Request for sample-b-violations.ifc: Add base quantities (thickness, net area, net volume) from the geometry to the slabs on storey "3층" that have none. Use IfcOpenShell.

First a look at what the model holds.

```python
import ifcopenshell
import ifcopenshell.util.element
import ifcopenshell.util.unit

model = ifcopenshell.open("sample-b-violations.ifc")
print(model.schema)
for unit_type in ("LENGTHUNIT", "AREAUNIT", "VOLUMEUNIT"):
    print(unit_type, ifcopenshell.util.unit.calculate_unit_scale(model, unit_type))
storey = next(s for s in model.by_type("IfcBuildingStorey") if s.Name == "3층")
slabs = [e for e in ifcopenshell.util.element.get_decomposition(storey) if e.is_a("IfcSlab")]
for e in sorted(slabs, key=lambda e: e.id()):
    print(e.id(), e.is_a(), e.Name, list(ifcopenshell.util.element.get_psets(e, qtos_only=True)), sep=" | ")
```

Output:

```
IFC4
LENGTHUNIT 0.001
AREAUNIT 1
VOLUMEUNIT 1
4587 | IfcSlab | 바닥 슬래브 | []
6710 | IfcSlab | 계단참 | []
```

```python
import ifcopenshell
import ifcopenshell.api.pset
import ifcopenshell.geom
import ifcopenshell.util.element
import ifcopenshell.util.shape
import ifcopenshell.util.unit

model = ifcopenshell.open("sample-b-violations.ifc")
unit_scale = ifcopenshell.util.unit.calculate_unit_scale(model)
area_scale = ifcopenshell.util.unit.calculate_unit_scale(model, "AREAUNIT")
volume_scale = ifcopenshell.util.unit.calculate_unit_scale(model, "VOLUMEUNIT")
settings = ifcopenshell.geom.settings()

storey = next(s for s in model.by_type("IfcBuildingStorey") if s.Name == "3층")
slabs = [e for e in ifcopenshell.util.element.get_decomposition(storey) if e.is_a("IfcSlab")]

for e in sorted(slabs, key=lambda e: e.id()):
    if ifcopenshell.util.element.get_psets(e, qtos_only=True, should_inherit=False):
        continue
    # Geometry comes back in metres, in the element's own axes.
    shape = ifcopenshell.geom.create_shape(settings, e)
    values = {
        "Width": ifcopenshell.util.shape.get_z(shape.geometry) / unit_scale,
        "NetArea": ifcopenshell.util.shape.get_footprint_area(shape.geometry) / area_scale,
        "NetVolume": ifcopenshell.util.shape.get_volume(shape.geometry) / volume_scale,
    }
    qto = ifcopenshell.api.pset.add_qto(model, product=e, name="Qto_SlabBaseQuantities")
    ifcopenshell.api.pset.edit_qto(model, qto=qto, properties=values)
    print(e.id(), {k: round(v, 3) for k, v in values.items()})

model.write("sample-b-violations_v2.ifc")
```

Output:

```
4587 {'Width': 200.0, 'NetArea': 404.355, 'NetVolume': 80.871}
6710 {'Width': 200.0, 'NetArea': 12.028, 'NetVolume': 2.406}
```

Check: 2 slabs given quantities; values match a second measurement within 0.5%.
